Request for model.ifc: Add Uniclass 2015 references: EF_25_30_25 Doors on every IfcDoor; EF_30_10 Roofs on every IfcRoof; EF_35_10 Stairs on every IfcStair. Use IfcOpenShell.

First a look at what the model holds.

```python
import ifcopenshell

model = ifcopenshell.open("model.ifc")
print(model.schema)
print("classifications:", [c.Name for c in model.by_type("IfcClassification")])
for ifc_class in ("IfcDoor", "IfcRoof", "IfcStair", "IfcWall", "IfcWindow"):
    print(ifc_class, len(model.by_type(ifc_class)))
```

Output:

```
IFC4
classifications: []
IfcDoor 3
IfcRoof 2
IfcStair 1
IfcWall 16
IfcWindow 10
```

```python
import ifcopenshell
import ifcopenshell.api.classification

model = ifcopenshell.open("model.ifc")

system = ifcopenshell.api.classification.add_classification(model, classification="Uniclass 2015")

codes = {
    "IfcDoor": ("EF_25_30_25", "Doors"),
    "IfcRoof": ("EF_30_10", "Roofs"),
    "IfcStair": ("EF_35_10", "Stairs"),
}
for ifc_class, (code, name) in codes.items():
    products = model.by_type(ifc_class)
    ifcopenshell.api.classification.add_reference(
        model, products=products, classification=system, identification=code, name=name
    )
    print(code, len(products))

model.write("model_updated.ifc")
```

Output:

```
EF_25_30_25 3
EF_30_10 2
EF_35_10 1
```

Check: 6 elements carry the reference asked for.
